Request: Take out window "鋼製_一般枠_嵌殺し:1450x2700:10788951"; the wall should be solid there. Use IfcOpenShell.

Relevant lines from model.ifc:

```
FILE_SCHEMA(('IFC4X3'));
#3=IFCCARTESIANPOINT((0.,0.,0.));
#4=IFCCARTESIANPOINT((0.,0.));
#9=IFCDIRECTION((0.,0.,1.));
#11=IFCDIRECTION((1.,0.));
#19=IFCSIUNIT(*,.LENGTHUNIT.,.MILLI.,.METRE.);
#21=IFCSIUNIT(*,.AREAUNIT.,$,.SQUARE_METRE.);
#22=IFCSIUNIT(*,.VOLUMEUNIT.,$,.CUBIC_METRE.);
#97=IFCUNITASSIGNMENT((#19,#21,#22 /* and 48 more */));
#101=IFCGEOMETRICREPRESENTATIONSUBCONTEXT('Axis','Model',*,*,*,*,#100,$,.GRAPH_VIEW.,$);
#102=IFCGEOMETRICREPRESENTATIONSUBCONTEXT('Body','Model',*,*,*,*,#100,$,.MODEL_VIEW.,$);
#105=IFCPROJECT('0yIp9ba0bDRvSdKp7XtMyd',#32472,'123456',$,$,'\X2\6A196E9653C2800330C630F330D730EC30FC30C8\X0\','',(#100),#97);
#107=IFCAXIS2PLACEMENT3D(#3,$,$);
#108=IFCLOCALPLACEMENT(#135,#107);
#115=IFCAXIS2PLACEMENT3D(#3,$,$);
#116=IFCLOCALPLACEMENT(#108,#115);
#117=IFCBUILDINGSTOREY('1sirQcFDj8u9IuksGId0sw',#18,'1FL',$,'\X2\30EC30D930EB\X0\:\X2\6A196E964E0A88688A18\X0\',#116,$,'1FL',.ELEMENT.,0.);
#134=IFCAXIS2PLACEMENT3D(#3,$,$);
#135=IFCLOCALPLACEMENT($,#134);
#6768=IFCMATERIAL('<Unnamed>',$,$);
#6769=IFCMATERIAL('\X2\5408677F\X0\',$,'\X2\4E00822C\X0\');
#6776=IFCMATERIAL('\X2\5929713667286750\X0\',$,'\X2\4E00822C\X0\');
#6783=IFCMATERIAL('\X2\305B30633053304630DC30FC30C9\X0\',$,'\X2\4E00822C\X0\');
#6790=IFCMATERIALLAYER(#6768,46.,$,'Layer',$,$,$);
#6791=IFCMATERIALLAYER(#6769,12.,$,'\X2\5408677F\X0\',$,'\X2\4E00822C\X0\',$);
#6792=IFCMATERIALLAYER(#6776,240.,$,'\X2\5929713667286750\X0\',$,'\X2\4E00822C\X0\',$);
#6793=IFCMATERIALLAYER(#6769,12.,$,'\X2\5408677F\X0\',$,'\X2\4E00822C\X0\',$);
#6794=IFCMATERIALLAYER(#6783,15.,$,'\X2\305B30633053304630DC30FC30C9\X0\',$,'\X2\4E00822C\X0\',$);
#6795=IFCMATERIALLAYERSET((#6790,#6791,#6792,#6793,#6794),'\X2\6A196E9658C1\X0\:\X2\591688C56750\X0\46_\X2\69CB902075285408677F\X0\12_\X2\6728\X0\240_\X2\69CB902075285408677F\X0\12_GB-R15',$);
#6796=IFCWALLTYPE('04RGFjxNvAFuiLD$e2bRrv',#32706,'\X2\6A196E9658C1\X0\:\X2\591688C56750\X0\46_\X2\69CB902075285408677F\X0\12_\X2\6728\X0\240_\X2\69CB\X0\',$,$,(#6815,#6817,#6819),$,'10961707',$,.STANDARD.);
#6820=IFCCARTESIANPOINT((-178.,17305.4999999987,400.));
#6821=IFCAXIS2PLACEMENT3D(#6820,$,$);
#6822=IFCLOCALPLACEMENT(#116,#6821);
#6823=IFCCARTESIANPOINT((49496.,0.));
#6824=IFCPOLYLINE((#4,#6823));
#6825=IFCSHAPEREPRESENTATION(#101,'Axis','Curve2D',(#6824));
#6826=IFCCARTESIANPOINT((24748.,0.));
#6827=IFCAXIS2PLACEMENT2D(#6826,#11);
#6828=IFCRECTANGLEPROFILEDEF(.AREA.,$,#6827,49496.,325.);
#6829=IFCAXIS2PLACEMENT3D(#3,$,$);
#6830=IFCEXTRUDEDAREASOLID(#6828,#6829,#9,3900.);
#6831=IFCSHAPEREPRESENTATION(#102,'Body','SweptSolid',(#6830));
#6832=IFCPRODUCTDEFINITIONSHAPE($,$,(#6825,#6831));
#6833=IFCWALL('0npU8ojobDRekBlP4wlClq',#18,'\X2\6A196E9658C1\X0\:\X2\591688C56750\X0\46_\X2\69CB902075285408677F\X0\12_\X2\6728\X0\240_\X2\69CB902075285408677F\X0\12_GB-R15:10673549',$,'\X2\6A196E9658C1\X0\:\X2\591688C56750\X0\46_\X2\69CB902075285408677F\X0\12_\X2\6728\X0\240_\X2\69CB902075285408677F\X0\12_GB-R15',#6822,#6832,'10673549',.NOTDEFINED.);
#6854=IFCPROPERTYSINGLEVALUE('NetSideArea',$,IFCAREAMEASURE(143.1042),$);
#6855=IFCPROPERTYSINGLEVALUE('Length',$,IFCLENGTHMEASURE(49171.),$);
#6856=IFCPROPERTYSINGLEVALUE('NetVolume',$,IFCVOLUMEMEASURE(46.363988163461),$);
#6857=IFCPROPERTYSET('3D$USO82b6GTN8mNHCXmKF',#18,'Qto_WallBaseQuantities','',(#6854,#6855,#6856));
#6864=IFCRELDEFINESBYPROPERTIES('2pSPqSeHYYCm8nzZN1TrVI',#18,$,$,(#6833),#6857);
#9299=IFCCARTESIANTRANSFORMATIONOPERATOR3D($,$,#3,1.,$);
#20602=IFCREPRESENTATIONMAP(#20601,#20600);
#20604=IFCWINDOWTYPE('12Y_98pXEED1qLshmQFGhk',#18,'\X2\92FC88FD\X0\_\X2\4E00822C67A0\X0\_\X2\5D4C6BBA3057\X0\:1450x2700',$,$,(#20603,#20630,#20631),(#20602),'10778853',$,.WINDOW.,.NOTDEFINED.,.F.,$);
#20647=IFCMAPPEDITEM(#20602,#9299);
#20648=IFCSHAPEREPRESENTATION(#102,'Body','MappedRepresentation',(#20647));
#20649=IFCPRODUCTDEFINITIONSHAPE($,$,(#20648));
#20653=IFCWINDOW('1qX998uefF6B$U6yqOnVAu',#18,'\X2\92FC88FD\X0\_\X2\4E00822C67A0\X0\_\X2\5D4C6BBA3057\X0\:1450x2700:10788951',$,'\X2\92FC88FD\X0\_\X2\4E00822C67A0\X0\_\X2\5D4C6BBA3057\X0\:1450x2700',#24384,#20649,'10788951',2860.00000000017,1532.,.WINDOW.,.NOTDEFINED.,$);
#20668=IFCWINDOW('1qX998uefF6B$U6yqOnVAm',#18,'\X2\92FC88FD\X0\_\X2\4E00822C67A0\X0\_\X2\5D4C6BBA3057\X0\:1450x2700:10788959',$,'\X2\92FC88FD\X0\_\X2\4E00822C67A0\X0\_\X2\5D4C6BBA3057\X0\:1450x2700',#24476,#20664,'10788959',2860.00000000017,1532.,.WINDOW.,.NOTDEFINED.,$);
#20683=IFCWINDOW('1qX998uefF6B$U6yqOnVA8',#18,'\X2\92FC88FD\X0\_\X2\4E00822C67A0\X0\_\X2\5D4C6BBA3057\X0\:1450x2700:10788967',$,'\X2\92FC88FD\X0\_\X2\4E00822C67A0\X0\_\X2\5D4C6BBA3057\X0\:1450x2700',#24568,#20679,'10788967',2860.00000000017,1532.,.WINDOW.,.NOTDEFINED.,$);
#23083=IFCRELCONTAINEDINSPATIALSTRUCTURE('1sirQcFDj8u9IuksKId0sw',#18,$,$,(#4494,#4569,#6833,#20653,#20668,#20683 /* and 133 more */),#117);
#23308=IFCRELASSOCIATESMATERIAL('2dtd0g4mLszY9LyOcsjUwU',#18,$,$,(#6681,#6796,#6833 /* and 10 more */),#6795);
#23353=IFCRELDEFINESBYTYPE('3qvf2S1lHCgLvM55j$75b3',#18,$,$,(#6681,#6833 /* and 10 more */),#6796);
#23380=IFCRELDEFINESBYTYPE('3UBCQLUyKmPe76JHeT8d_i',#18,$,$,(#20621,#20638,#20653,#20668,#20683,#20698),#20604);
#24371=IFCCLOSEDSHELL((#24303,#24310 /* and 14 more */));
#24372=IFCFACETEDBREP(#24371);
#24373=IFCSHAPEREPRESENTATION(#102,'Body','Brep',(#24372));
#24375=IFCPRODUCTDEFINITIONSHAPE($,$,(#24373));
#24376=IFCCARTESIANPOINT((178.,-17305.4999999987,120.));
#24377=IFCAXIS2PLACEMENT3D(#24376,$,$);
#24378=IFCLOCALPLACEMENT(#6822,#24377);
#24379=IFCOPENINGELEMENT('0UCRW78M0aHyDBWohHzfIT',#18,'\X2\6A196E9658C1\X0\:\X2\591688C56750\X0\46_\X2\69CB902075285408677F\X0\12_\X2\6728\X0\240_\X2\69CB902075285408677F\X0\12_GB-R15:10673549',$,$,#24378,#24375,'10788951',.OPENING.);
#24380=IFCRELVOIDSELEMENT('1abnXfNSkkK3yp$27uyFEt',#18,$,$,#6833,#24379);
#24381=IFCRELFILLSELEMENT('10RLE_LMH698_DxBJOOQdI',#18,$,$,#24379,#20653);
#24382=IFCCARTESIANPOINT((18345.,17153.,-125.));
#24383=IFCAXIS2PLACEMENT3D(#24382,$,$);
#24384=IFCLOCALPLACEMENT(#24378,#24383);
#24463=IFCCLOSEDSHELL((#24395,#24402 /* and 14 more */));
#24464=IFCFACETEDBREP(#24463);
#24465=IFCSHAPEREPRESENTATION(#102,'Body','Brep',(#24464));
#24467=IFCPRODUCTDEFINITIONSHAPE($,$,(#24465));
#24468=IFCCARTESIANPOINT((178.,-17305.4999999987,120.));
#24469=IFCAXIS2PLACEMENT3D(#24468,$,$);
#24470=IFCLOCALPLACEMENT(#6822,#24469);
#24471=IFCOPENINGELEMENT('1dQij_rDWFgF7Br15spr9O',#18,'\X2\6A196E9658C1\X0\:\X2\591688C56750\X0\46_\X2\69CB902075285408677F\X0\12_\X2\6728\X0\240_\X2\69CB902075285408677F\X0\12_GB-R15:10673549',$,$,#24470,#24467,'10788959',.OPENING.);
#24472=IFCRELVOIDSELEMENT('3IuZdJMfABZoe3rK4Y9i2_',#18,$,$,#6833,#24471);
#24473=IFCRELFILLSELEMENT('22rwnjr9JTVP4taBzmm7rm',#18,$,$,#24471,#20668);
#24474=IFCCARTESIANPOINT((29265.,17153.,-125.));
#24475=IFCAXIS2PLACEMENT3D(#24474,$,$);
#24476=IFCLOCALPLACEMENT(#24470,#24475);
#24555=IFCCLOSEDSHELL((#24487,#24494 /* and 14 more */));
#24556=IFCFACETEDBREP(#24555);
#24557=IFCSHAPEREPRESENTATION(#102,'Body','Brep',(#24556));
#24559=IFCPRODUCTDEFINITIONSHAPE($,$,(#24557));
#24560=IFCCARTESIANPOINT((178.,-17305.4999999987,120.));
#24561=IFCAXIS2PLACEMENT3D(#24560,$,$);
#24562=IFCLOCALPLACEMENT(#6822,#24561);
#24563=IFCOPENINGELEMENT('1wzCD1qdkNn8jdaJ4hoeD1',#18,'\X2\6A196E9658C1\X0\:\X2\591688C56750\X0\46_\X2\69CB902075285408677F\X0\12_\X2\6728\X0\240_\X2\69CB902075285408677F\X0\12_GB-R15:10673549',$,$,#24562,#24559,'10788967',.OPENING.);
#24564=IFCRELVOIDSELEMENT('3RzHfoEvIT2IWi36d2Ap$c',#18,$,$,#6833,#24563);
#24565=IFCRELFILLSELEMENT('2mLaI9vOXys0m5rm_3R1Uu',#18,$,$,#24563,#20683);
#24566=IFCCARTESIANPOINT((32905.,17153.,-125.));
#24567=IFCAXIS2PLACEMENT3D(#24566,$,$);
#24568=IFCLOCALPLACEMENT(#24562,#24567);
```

```python
import ifcopenshell
import ifcopenshell.api.feature
import ifcopenshell.api.pset
import ifcopenshell.api.root
import ifcopenshell.geom
import ifcopenshell.util.element
import ifcopenshell.util.shape
import ifcopenshell.util.unit

model = ifcopenshell.open("model.ifc")
area_scale = ifcopenshell.util.unit.calculate_unit_scale(model, "AREAUNIT")
volume_scale = ifcopenshell.util.unit.calculate_unit_scale(model, "VOLUMEUNIT")
settings = ifcopenshell.geom.settings()


def volume(element):
    """Net volume in cubic metres, openings subtracted."""
    shape = ifcopenshell.geom.create_shape(settings, element)
    return ifcopenshell.util.shape.get_volume(shape.geometry)


window = model.by_id(20653)
opening = window.FillsVoids[0].RelatingOpeningElement
wall = opening.VoidsElements[0].RelatingBuildingElement
before = volume(wall)

ifcopenshell.api.root.remove_product(model, product=window)
ifcopenshell.api.feature.remove_feature(model, feature=opening)

after = volume(wall)
thickness = 0.325  # wall thickness in metres

# Update the wall's stored quantities.
pset = model.by_id(ifcopenshell.util.element.get_pset(wall, "Qto_WallBaseQuantities", should_inherit=False)["id"])
ifcopenshell.api.pset.edit_pset(model, pset=pset, properties={
    "NetSideArea": model.create_entity("IfcAreaMeasure", after / thickness / area_scale),
    "NetVolume": model.create_entity("IfcVolumeMeasure", after / volume_scale),
})

print(f"wall volume {before:.3f} -> {after:.3f} m3")

model.write("model-out.ifc")
```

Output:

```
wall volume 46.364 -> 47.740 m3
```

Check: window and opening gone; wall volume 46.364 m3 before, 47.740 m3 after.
